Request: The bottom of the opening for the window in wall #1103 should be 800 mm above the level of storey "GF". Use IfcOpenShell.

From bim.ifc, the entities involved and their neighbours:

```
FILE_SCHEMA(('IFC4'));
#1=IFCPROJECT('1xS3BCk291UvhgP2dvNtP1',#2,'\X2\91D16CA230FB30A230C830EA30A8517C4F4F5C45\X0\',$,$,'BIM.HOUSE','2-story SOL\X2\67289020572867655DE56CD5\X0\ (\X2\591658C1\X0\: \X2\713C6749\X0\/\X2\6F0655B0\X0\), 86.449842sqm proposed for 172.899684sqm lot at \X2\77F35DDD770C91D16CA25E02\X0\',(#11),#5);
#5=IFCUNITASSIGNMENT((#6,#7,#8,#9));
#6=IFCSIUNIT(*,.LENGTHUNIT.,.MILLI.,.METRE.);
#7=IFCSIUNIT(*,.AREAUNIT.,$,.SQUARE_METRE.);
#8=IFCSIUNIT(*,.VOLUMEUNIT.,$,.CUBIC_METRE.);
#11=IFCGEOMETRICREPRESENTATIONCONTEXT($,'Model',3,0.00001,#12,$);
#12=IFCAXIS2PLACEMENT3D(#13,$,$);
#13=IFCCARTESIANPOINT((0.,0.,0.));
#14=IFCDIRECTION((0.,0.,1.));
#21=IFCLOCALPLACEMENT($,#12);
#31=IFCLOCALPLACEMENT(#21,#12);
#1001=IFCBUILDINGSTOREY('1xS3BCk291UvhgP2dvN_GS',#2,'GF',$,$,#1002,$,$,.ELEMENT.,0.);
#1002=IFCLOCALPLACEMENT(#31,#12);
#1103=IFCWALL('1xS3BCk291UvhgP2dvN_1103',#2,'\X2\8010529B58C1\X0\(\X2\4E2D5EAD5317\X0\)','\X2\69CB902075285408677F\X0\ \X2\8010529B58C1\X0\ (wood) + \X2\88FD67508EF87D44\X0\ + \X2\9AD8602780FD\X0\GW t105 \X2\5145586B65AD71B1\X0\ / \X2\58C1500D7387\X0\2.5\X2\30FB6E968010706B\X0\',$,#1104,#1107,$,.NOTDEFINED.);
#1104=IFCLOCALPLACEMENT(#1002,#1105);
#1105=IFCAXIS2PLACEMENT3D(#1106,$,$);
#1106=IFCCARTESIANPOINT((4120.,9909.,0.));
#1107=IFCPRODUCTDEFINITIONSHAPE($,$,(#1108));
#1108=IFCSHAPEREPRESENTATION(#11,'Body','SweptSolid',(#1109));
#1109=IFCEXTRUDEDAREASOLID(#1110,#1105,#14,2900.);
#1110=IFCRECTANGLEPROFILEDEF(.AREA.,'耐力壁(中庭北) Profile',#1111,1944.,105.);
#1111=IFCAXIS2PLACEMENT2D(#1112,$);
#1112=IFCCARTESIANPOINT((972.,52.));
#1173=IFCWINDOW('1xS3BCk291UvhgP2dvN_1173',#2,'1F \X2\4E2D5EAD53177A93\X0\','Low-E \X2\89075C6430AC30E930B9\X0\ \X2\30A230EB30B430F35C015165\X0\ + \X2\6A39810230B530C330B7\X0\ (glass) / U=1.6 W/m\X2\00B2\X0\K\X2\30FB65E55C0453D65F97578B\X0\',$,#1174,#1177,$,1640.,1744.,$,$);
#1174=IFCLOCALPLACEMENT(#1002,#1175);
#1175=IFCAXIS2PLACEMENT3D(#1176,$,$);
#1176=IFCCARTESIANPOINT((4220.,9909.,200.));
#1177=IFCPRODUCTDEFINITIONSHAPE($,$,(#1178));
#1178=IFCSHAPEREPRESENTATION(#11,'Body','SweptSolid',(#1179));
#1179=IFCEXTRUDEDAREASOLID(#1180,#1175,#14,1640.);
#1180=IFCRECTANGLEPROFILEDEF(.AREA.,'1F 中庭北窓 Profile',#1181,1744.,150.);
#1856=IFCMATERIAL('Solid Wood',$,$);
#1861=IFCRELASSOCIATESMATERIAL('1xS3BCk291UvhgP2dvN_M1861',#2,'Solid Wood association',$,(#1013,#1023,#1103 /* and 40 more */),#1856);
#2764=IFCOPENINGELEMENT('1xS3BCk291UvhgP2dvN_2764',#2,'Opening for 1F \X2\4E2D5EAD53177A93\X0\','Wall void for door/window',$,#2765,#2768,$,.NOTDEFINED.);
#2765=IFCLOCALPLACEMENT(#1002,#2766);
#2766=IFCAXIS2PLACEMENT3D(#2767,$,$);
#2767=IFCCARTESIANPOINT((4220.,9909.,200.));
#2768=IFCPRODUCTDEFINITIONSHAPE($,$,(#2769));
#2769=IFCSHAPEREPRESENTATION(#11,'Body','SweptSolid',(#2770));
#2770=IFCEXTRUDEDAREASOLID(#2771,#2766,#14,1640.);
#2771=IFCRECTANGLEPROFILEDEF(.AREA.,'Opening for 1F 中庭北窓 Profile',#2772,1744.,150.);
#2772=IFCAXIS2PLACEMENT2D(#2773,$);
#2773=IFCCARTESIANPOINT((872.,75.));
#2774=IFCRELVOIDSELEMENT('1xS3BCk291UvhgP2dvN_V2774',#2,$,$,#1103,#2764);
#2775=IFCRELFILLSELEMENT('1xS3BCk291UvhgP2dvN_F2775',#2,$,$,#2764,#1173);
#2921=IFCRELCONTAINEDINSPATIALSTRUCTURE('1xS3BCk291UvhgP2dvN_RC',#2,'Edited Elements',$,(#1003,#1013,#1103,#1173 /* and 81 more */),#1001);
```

```python
import numpy as np
import ifcopenshell
import ifcopenshell.api.geometry
import ifcopenshell.geom
import ifcopenshell.util.element
import ifcopenshell.util.placement
import ifcopenshell.util.shape
import ifcopenshell.util.unit

model = ifcopenshell.open("bim.ifc")
unit_scale = ifcopenshell.util.unit.calculate_unit_scale(model)

window = model.by_guid("1xS3BCk291UvhgP2dvN_1173")
opening = window.FillsVoids[0].RelatingOpeningElement
storey = ifcopenshell.util.element.get_container(window, ifc_class="IfcBuildingStorey")
level = ifcopenshell.util.placement.get_local_placement(storey.ObjectPlacement)[2, 3]

# The opening's origin need not be at the sill, so measure its lowest point.
shape = ifcopenshell.geom.create_shape(ifcopenshell.geom.settings(), opening)
bottom = ifcopenshell.util.shape.get_shape_bottom_elevation(shape, shape.geometry) / unit_scale
dz = level + 0.8 / unit_scale - bottom

shift = np.array([0.0, 0.0, dz])
# The window is not placed relative to its opening, so move both.
for product in (opening, window):
    matrix = ifcopenshell.util.placement.get_local_placement(product.ObjectPlacement)
    matrix[:3, 3] += shift
    ifcopenshell.api.geometry.edit_object_placement(model, product=product, matrix=matrix, is_si=False)

print(f"moved by {dz * unit_scale:+.3f} m")

model.write("bim_edited.ifc")
```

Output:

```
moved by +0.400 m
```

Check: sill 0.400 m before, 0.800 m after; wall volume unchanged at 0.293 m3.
